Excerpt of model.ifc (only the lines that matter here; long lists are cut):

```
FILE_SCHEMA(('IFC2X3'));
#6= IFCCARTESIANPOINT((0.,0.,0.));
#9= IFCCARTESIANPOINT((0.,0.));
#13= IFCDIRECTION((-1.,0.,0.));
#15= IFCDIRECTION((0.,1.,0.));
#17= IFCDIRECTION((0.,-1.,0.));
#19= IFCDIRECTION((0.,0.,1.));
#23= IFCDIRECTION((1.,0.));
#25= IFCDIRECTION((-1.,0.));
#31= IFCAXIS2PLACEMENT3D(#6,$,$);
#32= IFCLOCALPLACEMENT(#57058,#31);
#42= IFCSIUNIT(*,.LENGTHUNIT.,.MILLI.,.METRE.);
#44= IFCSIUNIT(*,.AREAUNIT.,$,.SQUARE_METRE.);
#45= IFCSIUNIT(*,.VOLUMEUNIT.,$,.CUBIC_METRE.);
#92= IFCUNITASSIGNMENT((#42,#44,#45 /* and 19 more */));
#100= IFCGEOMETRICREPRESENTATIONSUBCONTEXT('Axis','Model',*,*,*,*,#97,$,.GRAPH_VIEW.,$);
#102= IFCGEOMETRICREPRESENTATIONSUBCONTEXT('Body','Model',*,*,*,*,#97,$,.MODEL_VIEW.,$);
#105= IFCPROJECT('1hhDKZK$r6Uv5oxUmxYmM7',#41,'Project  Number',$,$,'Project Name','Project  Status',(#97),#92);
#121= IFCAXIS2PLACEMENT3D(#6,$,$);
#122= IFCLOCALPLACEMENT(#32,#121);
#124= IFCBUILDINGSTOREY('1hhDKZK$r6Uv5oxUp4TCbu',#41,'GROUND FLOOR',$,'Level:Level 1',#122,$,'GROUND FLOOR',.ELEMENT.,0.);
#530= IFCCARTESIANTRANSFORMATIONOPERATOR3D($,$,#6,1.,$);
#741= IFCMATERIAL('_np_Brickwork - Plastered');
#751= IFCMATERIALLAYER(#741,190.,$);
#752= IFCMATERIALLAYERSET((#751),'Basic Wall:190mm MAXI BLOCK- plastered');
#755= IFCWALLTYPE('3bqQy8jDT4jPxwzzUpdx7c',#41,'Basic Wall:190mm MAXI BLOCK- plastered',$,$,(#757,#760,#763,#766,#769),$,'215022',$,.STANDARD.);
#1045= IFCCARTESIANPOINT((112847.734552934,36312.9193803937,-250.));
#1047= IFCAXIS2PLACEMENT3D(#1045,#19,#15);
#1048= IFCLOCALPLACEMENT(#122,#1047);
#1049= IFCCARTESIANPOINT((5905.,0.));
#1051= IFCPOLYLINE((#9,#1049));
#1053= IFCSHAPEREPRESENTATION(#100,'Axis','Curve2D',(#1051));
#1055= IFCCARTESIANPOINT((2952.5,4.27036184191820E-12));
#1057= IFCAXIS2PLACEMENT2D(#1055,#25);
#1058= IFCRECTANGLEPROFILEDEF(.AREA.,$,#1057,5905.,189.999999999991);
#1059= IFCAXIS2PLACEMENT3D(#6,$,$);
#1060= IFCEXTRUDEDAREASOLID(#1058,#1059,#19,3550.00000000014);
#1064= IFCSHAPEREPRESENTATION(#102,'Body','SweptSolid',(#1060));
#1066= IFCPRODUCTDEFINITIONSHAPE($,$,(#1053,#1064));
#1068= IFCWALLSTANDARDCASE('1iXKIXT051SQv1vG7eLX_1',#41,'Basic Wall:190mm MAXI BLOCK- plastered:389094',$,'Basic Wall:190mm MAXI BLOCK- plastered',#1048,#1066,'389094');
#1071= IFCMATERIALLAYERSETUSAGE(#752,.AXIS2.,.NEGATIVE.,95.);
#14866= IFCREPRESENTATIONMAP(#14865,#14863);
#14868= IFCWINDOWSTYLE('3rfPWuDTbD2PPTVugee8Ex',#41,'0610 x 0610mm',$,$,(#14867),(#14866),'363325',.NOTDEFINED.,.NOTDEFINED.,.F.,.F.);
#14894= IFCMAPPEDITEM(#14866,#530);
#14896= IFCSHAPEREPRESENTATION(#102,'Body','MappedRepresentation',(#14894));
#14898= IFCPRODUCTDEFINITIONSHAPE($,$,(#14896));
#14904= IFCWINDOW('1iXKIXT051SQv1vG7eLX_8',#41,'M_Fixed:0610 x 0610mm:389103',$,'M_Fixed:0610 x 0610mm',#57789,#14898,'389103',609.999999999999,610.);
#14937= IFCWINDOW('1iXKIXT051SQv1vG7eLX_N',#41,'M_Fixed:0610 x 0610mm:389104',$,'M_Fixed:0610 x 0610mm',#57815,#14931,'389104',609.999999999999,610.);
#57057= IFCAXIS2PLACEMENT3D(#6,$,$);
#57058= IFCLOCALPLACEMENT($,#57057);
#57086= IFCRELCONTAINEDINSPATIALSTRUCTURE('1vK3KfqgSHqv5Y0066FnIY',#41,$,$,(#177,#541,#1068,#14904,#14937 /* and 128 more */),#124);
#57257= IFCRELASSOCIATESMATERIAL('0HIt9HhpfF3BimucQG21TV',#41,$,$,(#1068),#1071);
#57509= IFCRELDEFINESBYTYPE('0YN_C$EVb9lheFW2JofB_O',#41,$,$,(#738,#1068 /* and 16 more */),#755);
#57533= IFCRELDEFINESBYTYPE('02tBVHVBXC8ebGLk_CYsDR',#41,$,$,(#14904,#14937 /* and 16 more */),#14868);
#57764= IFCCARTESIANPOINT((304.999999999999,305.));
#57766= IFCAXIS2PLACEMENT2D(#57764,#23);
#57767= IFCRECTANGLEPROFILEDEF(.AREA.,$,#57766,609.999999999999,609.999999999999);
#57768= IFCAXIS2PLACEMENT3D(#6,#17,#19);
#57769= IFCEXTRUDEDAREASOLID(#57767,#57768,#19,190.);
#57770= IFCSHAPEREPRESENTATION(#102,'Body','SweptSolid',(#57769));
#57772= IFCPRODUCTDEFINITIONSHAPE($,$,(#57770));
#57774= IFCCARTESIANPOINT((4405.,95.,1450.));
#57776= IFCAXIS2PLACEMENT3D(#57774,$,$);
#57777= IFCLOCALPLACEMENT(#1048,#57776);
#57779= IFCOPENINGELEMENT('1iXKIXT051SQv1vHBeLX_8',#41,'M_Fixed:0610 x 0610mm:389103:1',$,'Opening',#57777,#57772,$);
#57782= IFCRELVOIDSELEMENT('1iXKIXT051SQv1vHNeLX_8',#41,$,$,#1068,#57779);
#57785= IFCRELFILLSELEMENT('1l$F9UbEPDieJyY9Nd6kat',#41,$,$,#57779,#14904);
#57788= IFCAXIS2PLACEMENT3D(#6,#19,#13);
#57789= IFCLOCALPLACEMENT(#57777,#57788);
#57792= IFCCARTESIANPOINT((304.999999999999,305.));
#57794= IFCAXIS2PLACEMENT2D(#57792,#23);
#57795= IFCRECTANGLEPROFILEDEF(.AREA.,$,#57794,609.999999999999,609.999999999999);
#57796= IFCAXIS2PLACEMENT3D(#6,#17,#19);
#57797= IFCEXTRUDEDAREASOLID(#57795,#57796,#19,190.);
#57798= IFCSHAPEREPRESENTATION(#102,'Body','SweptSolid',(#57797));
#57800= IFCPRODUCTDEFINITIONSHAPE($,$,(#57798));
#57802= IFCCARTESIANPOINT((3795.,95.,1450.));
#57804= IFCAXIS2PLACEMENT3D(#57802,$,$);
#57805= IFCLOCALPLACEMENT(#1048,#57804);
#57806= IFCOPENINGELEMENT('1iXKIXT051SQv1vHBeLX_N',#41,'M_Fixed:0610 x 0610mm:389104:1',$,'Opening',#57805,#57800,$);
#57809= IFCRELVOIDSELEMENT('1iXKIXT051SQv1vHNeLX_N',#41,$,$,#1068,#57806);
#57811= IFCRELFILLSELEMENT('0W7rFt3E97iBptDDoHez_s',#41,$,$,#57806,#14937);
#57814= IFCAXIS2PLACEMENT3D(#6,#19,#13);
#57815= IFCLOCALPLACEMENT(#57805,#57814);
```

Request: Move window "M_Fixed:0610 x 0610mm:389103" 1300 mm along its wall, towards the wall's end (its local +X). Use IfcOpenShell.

```python
import ifcopenshell
import ifcopenshell.api.geometry
import ifcopenshell.util.placement

model = ifcopenshell.open("model.ifc")

window = model.by_guid("1iXKIXT051SQv1vG7eLX_8")
opening = window.FillsVoids[0].RelatingOpeningElement
wall = opening.VoidsElements[0].RelatingBuildingElement

wall_matrix = ifcopenshell.util.placement.get_local_placement(wall.ObjectPlacement)
shift = wall_matrix[:3, 0] * 1300.0
before = ifcopenshell.util.placement.get_local_placement(window.ObjectPlacement)[:3, 3].copy()

# The window is placed relative to its opening, so it follows when the opening moves.
matrix = ifcopenshell.util.placement.get_local_placement(opening.ObjectPlacement)
matrix[:3, 3] += shift
ifcopenshell.api.geometry.edit_object_placement(
    model, product=opening, matrix=matrix, is_si=False, should_transform_children=True
)

after = ifcopenshell.util.placement.get_local_placement(window.ObjectPlacement)[:3, 3]
print("window moved by", (after - before).round(3) + 0.0)

model.write("model_updated.ifc")
```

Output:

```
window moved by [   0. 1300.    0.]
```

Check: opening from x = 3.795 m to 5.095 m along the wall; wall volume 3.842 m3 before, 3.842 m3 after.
